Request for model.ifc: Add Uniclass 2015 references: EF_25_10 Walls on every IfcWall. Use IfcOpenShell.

First a look at what the model holds.

```python
import ifcopenshell

model = ifcopenshell.open("model.ifc")
print(model.schema)
print("classifications:", [c.Name for c in model.by_type("IfcClassification")])
for ifc_class in ("IfcDoor", "IfcRoof", "IfcStair", "IfcWall", "IfcWindow"):
    print(ifc_class, len(model.by_type(ifc_class)))
```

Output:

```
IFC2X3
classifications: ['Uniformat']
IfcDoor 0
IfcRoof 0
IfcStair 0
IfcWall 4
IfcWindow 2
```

```python
import ifcopenshell
import ifcopenshell.api.classification

model = ifcopenshell.open("model.ifc")

# IFC2X3 requires Source and Edition and has no link from the project to the system.
system = model.create_entity("IfcClassification", Source="NBS", Edition="2015", Name="Uniclass 2015")

codes = {
    "IfcWall": ("EF_25_10", "Walls"),
}
for ifc_class, (code, name) in codes.items():
    products = model.by_type(ifc_class)
    ifcopenshell.api.classification.add_reference(
        model, products=products, classification=system, identification=code, name=name
    )
    print(code, len(products))

model.write("model_v2.ifc")
```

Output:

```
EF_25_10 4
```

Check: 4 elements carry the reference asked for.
